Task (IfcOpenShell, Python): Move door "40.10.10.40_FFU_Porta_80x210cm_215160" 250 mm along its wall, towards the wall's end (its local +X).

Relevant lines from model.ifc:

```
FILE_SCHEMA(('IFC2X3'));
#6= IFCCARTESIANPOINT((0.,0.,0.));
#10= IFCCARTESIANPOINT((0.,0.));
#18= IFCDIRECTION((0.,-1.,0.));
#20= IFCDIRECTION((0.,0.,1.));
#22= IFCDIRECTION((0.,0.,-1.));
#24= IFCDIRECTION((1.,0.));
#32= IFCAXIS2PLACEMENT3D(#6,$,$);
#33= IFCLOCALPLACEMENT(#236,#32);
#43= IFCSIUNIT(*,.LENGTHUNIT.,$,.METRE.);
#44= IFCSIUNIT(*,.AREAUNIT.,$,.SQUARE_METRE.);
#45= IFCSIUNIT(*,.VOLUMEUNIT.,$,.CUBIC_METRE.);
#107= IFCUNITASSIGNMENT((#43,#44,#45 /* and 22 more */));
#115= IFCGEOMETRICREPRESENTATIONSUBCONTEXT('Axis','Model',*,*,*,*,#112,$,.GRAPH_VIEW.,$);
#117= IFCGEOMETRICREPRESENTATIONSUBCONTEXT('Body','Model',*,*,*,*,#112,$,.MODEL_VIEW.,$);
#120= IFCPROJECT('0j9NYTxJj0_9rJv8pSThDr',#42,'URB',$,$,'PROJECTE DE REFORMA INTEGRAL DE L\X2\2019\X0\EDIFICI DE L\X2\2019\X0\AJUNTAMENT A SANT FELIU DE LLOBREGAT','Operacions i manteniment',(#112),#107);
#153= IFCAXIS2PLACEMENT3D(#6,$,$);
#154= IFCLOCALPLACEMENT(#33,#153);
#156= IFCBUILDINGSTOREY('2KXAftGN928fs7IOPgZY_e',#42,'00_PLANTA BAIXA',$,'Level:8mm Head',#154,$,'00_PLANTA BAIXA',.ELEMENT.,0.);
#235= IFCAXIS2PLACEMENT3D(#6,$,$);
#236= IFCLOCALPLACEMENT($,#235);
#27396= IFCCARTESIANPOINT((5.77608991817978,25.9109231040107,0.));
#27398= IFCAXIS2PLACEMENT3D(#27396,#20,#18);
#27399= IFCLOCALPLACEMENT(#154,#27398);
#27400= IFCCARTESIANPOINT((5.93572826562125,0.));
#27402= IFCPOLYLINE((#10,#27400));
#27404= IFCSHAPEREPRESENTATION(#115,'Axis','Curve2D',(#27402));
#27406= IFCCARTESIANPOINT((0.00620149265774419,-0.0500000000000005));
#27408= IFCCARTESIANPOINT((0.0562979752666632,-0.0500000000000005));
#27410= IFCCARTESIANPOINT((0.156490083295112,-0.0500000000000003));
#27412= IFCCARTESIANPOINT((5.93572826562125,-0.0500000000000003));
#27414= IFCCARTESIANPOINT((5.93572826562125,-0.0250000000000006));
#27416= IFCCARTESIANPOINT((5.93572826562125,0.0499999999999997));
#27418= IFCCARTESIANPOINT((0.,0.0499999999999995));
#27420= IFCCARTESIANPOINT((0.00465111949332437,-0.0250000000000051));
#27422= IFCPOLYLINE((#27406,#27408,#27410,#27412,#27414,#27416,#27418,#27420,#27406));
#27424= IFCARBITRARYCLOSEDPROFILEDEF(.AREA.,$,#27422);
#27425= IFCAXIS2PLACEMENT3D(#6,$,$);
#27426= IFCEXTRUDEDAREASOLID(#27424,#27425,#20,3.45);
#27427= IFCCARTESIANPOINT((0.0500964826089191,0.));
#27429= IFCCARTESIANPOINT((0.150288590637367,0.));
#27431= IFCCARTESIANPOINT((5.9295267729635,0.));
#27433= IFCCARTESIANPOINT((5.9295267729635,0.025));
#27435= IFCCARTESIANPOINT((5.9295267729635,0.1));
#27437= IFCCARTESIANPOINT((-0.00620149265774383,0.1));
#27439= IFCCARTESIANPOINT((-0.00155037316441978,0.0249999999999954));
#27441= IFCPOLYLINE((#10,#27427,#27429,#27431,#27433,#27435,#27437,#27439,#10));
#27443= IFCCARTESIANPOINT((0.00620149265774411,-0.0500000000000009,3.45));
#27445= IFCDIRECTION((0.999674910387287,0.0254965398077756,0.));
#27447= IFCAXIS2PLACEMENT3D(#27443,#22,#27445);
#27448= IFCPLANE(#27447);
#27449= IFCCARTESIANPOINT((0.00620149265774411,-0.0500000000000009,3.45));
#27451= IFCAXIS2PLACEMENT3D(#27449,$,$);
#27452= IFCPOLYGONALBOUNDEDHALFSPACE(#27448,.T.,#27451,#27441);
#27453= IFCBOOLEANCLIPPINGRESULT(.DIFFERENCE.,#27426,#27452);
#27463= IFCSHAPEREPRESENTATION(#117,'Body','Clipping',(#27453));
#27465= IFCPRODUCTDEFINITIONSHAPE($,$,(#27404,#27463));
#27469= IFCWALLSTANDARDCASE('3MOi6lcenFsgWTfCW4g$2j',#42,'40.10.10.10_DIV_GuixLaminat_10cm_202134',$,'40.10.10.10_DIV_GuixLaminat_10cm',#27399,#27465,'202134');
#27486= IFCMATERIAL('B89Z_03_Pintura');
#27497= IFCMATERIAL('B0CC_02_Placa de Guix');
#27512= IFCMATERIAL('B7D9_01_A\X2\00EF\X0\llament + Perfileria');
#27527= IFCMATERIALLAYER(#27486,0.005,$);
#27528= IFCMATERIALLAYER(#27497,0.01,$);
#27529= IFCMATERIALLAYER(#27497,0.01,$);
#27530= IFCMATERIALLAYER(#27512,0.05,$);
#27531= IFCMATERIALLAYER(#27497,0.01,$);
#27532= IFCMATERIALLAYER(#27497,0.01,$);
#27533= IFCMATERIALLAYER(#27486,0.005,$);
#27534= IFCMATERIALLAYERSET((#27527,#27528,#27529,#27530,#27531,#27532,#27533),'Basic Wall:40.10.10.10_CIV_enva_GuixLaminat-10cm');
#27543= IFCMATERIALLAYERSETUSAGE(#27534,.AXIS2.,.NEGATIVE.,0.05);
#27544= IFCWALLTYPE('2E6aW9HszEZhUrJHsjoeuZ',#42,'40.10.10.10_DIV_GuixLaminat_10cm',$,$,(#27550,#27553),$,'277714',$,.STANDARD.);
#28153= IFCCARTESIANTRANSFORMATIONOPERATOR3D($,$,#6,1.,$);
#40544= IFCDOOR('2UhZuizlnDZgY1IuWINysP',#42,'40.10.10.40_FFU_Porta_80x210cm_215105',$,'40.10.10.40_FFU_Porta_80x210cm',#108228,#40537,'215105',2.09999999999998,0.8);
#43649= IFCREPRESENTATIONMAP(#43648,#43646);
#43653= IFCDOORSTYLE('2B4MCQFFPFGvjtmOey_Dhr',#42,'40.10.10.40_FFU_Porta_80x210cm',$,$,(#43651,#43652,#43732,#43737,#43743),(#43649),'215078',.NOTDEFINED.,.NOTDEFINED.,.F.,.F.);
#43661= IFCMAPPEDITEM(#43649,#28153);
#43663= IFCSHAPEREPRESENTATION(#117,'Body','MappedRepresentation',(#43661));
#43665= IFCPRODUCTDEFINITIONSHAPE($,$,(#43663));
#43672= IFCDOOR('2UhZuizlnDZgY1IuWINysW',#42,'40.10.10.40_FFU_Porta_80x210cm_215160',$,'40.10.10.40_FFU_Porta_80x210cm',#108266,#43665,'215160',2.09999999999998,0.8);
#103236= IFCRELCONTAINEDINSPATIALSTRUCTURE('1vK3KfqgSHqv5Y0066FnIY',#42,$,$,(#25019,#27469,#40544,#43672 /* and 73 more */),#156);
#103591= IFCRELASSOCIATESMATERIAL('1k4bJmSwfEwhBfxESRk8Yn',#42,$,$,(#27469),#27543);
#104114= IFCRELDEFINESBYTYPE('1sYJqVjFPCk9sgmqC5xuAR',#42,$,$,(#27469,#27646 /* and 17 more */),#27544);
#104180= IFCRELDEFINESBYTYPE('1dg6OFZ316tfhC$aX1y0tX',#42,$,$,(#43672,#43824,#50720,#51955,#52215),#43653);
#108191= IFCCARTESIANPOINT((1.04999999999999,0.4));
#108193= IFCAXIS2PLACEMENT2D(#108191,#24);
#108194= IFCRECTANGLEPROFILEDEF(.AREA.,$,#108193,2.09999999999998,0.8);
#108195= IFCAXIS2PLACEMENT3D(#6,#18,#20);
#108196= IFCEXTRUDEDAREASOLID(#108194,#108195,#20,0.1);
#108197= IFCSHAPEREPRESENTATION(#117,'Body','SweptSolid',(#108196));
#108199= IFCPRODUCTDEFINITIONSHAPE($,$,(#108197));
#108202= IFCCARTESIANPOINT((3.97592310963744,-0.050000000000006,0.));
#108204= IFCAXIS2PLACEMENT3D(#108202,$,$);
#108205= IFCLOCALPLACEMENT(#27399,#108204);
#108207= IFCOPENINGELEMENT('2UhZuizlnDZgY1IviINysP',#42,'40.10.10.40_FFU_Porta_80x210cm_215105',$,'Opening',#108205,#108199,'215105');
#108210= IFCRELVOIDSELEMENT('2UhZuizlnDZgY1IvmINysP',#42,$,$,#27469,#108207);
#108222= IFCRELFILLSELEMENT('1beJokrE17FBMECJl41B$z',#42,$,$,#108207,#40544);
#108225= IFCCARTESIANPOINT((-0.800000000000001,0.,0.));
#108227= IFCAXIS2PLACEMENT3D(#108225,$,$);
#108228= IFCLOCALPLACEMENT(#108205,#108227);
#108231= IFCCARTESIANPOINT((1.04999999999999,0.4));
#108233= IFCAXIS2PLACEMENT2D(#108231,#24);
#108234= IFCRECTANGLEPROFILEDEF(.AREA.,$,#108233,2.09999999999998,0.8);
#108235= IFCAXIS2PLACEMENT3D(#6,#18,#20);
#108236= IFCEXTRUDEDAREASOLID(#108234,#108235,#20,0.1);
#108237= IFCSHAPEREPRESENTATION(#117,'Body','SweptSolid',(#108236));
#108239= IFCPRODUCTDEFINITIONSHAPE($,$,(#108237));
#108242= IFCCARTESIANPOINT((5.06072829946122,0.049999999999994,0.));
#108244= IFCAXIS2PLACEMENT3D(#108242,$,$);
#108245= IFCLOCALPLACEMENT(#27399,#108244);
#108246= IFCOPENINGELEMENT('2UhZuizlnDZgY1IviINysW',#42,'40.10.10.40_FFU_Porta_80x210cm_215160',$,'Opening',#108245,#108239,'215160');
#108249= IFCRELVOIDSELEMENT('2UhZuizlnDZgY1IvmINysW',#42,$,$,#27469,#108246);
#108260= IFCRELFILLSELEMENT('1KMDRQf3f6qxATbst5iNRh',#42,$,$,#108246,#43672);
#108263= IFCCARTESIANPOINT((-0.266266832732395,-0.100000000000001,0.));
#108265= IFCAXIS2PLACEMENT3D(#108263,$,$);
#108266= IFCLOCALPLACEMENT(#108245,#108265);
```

```python
import ifcopenshell
import ifcopenshell.api.geometry
import ifcopenshell.util.placement

model = ifcopenshell.open("model.ifc")

door = model.by_guid("2UhZuizlnDZgY1IuWINysW")
opening = door.FillsVoids[0].RelatingOpeningElement
wall = opening.VoidsElements[0].RelatingBuildingElement

wall_matrix = ifcopenshell.util.placement.get_local_placement(wall.ObjectPlacement)
shift = wall_matrix[:3, 0] * 0.25
before = ifcopenshell.util.placement.get_local_placement(door.ObjectPlacement)[:3, 3].copy()

# The door is placed relative to its opening, so it follows when the opening moves.
matrix = ifcopenshell.util.placement.get_local_placement(opening.ObjectPlacement)
matrix[:3, 3] += shift
ifcopenshell.api.geometry.edit_object_placement(
    model, product=opening, matrix=matrix, is_si=False, should_transform_children=True
)

after = ifcopenshell.util.placement.get_local_placement(door.ObjectPlacement)[:3, 3]
print("door moved by", (after - before).round(3) + 0.0)

model.write("model_v2.ifc")
```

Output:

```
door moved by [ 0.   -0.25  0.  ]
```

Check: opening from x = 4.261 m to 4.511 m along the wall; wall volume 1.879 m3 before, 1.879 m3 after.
